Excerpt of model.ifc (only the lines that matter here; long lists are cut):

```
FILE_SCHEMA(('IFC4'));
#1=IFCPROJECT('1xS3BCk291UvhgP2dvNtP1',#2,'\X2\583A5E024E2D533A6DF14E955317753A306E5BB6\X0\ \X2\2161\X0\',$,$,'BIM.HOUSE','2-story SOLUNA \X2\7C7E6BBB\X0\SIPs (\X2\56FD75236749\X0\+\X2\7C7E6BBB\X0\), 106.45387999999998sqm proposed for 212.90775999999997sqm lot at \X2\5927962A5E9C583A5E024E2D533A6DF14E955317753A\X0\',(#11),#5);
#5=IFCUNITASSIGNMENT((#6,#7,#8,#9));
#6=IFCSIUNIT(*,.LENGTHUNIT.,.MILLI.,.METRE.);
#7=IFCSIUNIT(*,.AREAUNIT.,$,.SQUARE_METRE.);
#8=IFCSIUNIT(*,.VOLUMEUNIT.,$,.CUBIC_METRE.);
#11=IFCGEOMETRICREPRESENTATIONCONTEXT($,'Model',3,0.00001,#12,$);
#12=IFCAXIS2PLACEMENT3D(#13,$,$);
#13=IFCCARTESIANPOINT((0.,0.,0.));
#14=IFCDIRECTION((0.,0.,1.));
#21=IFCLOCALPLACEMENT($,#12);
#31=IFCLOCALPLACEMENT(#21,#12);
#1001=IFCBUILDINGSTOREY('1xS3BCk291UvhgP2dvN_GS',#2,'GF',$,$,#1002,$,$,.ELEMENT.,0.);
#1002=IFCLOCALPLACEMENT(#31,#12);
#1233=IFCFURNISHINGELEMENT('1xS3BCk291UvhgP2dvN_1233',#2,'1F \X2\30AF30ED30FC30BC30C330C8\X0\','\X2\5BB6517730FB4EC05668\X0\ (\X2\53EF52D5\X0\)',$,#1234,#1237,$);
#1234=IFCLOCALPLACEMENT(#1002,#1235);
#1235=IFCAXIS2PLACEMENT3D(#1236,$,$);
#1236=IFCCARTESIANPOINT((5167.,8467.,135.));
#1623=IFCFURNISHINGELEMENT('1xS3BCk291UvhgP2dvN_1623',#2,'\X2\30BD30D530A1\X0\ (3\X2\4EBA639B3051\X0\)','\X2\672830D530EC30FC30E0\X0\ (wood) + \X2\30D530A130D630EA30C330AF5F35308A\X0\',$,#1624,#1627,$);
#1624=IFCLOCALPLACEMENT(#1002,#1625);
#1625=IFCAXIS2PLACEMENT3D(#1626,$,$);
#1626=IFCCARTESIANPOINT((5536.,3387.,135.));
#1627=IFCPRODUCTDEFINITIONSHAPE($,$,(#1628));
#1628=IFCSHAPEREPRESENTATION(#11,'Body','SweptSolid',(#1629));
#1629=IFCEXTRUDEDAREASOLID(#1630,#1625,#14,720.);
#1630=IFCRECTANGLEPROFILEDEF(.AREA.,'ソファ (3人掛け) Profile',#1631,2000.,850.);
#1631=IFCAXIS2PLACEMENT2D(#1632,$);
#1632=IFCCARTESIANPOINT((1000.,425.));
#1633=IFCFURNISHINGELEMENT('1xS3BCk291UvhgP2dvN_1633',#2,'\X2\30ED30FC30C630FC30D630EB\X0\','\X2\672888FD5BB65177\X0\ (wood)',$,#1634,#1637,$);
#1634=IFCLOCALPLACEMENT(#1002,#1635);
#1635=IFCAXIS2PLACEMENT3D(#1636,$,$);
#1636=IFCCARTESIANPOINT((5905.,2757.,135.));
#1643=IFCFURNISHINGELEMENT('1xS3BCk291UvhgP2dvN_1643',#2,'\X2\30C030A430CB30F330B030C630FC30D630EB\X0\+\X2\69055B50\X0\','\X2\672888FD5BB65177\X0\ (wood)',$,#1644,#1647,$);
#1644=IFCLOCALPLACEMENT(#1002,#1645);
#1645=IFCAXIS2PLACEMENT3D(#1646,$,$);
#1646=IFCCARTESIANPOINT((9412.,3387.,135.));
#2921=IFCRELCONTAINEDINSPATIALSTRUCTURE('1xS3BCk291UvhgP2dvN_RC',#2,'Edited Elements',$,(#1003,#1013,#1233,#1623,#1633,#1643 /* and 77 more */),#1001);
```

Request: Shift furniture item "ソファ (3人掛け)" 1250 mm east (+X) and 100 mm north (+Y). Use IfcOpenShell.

```python
import ifcopenshell
import ifcopenshell.api.geometry
import ifcopenshell.util.placement

model = ifcopenshell.open("model.ifc")

item = model.by_id(1623)
matrix = ifcopenshell.util.placement.get_local_placement(item.ObjectPlacement)
matrix[0, 3] += 1250.0
matrix[1, 3] += 100.0
ifcopenshell.api.geometry.edit_object_placement(model, product=item, matrix=matrix, is_si=False)

print(ifcopenshell.util.placement.get_local_placement(item.ObjectPlacement).round(3) + 0.0)

model.write("model_updated.ifc")
```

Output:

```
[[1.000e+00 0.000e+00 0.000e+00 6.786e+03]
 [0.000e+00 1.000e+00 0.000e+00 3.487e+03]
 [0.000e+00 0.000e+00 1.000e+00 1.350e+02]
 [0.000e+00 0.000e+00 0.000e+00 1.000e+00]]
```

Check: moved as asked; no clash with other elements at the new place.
